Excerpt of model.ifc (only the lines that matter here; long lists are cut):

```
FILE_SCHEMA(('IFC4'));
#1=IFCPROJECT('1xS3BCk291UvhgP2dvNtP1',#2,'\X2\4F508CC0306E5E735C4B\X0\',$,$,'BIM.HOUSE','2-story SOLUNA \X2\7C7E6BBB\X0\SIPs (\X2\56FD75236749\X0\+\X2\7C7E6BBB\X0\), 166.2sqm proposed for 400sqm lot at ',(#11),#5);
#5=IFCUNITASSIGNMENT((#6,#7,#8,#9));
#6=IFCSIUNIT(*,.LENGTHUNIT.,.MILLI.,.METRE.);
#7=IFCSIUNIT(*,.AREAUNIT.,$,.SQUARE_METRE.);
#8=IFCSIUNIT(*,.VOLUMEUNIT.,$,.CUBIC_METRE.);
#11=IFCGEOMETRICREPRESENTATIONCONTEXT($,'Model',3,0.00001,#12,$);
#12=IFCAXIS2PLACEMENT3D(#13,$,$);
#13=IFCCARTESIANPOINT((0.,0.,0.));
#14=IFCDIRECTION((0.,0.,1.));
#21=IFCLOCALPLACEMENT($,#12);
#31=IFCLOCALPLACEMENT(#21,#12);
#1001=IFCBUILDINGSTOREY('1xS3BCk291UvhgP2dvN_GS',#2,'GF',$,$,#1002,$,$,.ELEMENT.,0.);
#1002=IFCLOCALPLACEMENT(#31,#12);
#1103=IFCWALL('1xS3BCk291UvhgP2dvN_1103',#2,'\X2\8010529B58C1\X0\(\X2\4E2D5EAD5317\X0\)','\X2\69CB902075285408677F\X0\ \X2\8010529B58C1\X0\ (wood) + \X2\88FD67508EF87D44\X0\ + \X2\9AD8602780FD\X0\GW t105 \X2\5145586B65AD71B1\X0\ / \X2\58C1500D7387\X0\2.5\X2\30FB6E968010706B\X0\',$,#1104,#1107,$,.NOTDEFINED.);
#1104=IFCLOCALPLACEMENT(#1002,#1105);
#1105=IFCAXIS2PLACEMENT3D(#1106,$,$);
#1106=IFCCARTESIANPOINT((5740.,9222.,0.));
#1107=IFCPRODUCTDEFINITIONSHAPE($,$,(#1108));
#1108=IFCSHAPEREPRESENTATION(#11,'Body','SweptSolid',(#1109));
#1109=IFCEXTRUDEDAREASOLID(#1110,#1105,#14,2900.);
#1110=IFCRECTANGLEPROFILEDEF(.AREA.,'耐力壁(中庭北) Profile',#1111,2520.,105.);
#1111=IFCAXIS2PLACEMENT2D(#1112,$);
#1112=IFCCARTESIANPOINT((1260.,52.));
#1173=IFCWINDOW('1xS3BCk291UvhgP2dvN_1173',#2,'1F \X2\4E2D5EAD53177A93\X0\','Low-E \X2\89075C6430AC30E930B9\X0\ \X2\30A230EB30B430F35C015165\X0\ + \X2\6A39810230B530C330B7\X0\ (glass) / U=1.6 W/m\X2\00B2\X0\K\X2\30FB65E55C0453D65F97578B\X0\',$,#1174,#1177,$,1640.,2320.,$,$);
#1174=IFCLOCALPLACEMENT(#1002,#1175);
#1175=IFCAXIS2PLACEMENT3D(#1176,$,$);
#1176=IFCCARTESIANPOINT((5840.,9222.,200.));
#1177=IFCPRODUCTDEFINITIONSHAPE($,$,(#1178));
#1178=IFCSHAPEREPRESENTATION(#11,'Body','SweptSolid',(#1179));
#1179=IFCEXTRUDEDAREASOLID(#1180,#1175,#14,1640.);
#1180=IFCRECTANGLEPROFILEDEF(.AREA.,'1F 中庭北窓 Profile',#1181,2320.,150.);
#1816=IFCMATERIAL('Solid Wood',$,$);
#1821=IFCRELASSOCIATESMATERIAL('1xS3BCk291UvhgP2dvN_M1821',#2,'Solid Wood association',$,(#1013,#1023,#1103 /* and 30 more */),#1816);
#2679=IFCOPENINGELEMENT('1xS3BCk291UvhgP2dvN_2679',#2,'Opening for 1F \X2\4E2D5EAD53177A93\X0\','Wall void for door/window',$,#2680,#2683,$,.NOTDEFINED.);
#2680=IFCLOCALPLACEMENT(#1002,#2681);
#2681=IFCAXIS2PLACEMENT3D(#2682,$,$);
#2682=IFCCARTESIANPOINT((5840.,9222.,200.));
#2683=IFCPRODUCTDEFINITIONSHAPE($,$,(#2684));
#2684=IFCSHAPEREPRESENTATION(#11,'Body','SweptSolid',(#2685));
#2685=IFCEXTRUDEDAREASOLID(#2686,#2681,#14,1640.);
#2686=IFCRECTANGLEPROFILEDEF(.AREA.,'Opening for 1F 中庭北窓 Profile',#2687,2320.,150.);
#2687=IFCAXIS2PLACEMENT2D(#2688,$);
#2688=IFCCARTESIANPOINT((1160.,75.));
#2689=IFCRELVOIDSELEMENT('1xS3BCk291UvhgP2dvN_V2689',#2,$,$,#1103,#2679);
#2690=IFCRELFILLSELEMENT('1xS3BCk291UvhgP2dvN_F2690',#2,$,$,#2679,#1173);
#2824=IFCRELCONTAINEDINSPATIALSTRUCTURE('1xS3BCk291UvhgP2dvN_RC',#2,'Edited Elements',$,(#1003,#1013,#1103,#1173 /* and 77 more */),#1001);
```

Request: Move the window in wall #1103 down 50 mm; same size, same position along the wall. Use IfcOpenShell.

```python
import numpy as np
import ifcopenshell
import ifcopenshell.api.geometry
import ifcopenshell.util.placement
import ifcopenshell.util.unit

model = ifcopenshell.open("model.ifc")
unit_scale = ifcopenshell.util.unit.calculate_unit_scale(model)

window = model.by_guid("1xS3BCk291UvhgP2dvN_1173")
opening = window.FillsVoids[0].RelatingOpeningElement
dz = -0.05 / unit_scale

shift = np.array([0.0, 0.0, dz])
# The window is not placed relative to its opening, so move both.
for product in (opening, window):
    matrix = ifcopenshell.util.placement.get_local_placement(product.ObjectPlacement)
    matrix[:3, 3] += shift
    ifcopenshell.api.geometry.edit_object_placement(model, product=product, matrix=matrix, is_si=False)

print(f"moved by {dz * unit_scale:+.3f} m")

model.write("model_v2.ifc")
```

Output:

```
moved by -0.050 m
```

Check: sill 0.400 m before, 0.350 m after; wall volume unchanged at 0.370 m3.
